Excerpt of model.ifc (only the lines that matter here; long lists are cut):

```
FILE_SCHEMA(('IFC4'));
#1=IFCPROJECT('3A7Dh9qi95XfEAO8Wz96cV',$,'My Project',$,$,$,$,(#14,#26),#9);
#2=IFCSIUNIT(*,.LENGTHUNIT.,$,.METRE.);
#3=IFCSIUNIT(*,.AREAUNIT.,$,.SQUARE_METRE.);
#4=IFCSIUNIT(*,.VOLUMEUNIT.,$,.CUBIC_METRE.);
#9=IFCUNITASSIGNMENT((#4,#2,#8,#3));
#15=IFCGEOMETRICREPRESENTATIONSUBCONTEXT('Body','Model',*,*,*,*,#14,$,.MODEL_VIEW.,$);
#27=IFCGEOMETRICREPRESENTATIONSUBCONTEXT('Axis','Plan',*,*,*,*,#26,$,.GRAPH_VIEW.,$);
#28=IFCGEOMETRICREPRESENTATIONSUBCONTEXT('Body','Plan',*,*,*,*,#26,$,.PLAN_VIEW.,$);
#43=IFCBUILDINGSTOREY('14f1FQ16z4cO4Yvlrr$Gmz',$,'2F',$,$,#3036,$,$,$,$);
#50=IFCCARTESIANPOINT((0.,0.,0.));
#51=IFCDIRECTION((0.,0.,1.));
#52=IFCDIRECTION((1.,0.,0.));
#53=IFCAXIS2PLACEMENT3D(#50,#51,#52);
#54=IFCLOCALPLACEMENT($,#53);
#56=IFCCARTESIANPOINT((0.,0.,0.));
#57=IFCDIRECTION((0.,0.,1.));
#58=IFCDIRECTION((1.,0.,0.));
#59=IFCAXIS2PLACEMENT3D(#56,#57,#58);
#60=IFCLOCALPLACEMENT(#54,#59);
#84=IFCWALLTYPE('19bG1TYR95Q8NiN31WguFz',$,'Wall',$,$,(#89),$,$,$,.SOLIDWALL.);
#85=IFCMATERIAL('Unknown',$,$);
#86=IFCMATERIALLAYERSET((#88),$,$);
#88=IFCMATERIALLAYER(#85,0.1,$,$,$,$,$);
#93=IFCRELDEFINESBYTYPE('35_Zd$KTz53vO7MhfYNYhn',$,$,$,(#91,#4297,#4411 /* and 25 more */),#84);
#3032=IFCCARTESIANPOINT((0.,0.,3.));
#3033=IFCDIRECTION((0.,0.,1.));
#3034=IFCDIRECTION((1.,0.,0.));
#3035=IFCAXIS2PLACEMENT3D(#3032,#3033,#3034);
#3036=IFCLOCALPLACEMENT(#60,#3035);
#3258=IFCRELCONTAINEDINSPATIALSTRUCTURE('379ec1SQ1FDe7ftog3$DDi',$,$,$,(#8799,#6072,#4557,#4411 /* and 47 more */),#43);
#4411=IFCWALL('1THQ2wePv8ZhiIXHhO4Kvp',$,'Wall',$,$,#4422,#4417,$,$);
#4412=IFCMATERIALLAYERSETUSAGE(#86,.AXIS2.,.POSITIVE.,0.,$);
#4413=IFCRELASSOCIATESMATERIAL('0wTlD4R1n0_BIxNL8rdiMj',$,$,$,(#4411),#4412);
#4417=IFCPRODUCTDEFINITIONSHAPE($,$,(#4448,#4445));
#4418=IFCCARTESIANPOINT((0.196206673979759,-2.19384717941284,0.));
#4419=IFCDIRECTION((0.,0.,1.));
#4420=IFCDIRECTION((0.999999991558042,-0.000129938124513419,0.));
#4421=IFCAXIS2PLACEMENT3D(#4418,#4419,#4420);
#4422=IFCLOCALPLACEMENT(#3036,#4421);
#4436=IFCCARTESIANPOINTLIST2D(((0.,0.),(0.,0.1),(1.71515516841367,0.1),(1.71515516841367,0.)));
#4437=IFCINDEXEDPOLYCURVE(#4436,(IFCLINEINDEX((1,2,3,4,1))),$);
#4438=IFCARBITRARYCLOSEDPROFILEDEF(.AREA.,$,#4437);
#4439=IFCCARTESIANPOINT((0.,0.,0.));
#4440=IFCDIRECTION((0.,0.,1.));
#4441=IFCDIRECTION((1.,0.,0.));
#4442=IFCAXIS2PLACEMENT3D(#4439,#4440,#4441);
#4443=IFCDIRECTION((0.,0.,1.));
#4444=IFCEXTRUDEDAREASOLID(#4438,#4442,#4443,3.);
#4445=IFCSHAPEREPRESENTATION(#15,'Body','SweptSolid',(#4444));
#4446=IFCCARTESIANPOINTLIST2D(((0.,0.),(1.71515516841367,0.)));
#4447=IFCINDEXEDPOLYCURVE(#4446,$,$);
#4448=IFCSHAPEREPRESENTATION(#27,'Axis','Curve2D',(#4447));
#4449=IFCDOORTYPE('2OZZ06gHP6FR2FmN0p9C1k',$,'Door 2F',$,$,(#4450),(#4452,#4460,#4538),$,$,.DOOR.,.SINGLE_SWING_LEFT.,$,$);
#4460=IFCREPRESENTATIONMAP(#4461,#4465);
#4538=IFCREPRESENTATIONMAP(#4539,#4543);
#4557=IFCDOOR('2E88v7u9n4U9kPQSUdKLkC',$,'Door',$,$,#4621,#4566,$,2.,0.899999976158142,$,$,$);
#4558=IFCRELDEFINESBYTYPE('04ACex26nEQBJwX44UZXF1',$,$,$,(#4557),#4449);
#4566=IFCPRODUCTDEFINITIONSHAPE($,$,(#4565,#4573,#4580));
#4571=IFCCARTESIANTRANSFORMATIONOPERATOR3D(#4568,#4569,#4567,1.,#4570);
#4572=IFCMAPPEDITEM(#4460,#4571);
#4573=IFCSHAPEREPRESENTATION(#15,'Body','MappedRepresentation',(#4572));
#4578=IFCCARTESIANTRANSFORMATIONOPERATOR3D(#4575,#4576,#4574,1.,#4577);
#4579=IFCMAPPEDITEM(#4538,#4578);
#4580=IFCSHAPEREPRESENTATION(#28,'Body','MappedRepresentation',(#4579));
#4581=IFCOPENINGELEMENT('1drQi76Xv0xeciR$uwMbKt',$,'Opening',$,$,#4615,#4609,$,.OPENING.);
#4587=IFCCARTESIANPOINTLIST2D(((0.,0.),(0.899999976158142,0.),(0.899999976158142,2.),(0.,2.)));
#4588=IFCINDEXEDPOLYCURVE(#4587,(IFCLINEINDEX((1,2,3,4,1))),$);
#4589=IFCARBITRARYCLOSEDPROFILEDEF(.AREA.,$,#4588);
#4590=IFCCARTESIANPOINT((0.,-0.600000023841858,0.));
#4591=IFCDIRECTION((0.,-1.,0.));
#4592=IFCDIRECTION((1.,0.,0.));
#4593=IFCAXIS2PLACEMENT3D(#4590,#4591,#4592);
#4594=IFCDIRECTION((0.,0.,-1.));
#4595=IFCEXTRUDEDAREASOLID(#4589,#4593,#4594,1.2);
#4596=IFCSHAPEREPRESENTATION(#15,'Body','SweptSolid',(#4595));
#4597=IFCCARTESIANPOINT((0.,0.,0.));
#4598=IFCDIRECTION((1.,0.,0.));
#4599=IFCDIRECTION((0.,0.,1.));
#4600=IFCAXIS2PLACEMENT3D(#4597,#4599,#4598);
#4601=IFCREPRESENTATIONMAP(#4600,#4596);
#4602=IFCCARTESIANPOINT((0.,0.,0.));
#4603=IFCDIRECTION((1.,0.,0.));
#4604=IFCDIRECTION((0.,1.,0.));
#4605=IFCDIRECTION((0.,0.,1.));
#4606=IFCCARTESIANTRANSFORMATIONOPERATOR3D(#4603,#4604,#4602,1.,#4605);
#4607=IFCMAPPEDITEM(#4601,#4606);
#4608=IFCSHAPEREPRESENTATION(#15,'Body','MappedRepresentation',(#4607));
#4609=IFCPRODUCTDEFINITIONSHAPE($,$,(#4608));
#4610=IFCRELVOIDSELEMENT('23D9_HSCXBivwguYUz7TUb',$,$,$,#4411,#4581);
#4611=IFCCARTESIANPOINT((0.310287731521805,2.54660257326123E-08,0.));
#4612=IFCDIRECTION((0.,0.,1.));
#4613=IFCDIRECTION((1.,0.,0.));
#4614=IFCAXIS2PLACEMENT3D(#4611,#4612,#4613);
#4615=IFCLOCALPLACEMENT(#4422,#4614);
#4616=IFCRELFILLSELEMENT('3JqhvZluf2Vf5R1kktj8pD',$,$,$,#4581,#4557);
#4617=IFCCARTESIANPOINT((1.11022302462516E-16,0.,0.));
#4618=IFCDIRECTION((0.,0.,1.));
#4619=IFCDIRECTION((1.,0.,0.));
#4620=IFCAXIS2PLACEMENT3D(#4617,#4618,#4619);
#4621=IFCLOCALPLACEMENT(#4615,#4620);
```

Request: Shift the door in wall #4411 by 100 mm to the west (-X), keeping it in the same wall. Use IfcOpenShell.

```python
import ifcopenshell
import ifcopenshell.api.geometry
import ifcopenshell.util.placement

model = ifcopenshell.open("model.ifc")

door = model.by_guid("2E88v7u9n4U9kPQSUdKLkC")
opening = door.FillsVoids[0].RelatingOpeningElement
wall = opening.VoidsElements[0].RelatingBuildingElement

wall_matrix = ifcopenshell.util.placement.get_local_placement(wall.ObjectPlacement)
shift = wall_matrix[:3, 0] * -0.1
before = ifcopenshell.util.placement.get_local_placement(door.ObjectPlacement)[:3, 3].copy()

# The door is placed relative to its opening, so it follows when the opening moves.
matrix = ifcopenshell.util.placement.get_local_placement(opening.ObjectPlacement)
matrix[:3, 3] += shift
ifcopenshell.api.geometry.edit_object_placement(
    model, product=opening, matrix=matrix, is_si=False, should_transform_children=True
)

after = ifcopenshell.util.placement.get_local_placement(door.ObjectPlacement)[:3, 3]
print("door moved by", (after - before).round(3) + 0.0)

model.write("model_edited.ifc")
```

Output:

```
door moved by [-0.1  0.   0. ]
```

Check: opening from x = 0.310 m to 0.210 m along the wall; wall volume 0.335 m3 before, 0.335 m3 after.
